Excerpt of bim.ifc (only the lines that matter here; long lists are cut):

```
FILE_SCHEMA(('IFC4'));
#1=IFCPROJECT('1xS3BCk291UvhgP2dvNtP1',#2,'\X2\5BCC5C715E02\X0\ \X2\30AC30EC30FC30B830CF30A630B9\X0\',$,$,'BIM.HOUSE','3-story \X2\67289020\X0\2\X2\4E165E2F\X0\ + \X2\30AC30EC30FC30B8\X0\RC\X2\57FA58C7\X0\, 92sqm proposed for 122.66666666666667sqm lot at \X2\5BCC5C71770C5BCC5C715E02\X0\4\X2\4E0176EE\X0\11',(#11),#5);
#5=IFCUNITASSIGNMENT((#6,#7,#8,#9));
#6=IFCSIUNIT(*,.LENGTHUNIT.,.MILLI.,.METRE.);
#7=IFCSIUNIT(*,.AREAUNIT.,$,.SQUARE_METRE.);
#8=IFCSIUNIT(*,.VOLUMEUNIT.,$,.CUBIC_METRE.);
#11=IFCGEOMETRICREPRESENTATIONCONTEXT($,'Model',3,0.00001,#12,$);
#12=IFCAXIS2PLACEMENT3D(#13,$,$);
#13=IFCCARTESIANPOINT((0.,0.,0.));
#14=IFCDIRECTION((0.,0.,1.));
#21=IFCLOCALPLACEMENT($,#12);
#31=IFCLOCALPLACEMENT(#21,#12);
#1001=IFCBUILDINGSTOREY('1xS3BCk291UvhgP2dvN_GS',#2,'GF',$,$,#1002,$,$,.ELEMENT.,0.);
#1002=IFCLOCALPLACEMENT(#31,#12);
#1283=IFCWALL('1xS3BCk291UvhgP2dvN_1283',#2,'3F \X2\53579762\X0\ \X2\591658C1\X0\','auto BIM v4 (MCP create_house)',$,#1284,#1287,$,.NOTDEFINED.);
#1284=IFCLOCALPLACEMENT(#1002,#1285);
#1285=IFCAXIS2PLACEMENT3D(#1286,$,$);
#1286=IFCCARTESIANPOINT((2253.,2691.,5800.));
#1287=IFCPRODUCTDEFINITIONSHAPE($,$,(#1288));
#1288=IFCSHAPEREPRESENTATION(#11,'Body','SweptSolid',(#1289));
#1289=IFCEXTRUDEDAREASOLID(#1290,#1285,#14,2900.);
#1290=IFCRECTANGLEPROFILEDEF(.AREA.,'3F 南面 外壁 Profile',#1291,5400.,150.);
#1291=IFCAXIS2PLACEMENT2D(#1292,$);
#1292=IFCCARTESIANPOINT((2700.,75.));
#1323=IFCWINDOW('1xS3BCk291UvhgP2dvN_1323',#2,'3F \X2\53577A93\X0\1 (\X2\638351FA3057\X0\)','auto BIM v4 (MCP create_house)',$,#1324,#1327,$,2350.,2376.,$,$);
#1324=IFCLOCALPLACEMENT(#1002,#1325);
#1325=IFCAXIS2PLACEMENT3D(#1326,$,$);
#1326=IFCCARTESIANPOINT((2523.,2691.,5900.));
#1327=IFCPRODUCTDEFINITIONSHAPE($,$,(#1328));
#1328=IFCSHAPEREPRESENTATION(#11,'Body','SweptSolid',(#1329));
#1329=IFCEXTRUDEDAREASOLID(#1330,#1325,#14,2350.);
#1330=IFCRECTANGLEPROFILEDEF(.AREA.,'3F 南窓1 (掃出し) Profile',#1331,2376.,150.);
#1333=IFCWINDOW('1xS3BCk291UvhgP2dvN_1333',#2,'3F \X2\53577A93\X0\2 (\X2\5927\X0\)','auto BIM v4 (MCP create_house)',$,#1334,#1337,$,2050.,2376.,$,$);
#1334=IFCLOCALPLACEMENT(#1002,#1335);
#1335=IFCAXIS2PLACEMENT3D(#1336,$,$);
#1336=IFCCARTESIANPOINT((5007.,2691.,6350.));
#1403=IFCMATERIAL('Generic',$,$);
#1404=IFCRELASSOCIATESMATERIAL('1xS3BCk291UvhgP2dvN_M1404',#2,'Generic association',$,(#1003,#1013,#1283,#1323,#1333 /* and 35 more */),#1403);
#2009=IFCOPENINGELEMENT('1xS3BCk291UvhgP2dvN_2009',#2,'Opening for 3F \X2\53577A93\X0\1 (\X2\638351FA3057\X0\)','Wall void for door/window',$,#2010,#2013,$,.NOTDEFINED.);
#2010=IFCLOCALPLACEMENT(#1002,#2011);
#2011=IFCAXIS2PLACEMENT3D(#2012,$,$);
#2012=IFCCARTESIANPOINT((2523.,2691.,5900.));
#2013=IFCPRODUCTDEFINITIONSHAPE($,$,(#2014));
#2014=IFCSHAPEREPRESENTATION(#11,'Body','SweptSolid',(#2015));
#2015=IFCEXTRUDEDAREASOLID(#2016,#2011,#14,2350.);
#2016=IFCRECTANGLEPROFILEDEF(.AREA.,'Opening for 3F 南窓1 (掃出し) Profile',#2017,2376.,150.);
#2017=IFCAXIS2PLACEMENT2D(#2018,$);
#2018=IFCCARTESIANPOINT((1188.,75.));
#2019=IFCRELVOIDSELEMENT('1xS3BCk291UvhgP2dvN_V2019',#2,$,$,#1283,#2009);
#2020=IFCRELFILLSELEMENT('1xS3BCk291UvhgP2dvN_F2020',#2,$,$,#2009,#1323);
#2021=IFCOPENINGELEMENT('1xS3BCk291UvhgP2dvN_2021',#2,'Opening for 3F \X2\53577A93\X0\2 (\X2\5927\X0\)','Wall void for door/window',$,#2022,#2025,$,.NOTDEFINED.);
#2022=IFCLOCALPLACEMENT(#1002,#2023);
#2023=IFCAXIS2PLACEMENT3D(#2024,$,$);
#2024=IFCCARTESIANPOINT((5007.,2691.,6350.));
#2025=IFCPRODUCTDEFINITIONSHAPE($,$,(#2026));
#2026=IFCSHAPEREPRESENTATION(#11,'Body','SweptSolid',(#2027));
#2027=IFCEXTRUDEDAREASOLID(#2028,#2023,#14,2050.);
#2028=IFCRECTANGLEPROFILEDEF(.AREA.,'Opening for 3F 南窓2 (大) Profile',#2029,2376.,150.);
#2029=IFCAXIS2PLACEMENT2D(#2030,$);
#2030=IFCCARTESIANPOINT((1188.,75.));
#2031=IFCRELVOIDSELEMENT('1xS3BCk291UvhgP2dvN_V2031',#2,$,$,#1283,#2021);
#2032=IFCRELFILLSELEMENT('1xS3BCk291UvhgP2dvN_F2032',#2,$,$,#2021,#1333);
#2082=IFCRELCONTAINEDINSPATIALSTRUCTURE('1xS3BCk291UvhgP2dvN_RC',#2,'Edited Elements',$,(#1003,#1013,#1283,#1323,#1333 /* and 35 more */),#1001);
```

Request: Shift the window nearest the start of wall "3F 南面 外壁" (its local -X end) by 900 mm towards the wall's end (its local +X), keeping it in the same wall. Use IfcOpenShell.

```python
import ifcopenshell
import ifcopenshell.api.geometry
import ifcopenshell.util.placement
import ifcopenshell.util.unit

model = ifcopenshell.open("bim.ifc")
unit_scale = ifcopenshell.util.unit.calculate_unit_scale(model)

window = model.by_guid("1xS3BCk291UvhgP2dvN_1323")
opening = window.FillsVoids[0].RelatingOpeningElement
wall = opening.VoidsElements[0].RelatingBuildingElement

wall_matrix = ifcopenshell.util.placement.get_local_placement(wall.ObjectPlacement)
shift = wall_matrix[:3, 0] * 0.9 / unit_scale
before = ifcopenshell.util.placement.get_local_placement(window.ObjectPlacement)[:3, 3].copy()

# The window is not placed relative to its opening, so move both.
for product in (opening, window):
    matrix = ifcopenshell.util.placement.get_local_placement(product.ObjectPlacement)
    matrix[:3, 3] += shift
    ifcopenshell.api.geometry.edit_object_placement(model, product=product, matrix=matrix, is_si=False)

after = ifcopenshell.util.placement.get_local_placement(window.ObjectPlacement)[:3, 3]
print("window moved by", (after - before).round(3) + 0.0)

model.write("bim_edited.ifc")
```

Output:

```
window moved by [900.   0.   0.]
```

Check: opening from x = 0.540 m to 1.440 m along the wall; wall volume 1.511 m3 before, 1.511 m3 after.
